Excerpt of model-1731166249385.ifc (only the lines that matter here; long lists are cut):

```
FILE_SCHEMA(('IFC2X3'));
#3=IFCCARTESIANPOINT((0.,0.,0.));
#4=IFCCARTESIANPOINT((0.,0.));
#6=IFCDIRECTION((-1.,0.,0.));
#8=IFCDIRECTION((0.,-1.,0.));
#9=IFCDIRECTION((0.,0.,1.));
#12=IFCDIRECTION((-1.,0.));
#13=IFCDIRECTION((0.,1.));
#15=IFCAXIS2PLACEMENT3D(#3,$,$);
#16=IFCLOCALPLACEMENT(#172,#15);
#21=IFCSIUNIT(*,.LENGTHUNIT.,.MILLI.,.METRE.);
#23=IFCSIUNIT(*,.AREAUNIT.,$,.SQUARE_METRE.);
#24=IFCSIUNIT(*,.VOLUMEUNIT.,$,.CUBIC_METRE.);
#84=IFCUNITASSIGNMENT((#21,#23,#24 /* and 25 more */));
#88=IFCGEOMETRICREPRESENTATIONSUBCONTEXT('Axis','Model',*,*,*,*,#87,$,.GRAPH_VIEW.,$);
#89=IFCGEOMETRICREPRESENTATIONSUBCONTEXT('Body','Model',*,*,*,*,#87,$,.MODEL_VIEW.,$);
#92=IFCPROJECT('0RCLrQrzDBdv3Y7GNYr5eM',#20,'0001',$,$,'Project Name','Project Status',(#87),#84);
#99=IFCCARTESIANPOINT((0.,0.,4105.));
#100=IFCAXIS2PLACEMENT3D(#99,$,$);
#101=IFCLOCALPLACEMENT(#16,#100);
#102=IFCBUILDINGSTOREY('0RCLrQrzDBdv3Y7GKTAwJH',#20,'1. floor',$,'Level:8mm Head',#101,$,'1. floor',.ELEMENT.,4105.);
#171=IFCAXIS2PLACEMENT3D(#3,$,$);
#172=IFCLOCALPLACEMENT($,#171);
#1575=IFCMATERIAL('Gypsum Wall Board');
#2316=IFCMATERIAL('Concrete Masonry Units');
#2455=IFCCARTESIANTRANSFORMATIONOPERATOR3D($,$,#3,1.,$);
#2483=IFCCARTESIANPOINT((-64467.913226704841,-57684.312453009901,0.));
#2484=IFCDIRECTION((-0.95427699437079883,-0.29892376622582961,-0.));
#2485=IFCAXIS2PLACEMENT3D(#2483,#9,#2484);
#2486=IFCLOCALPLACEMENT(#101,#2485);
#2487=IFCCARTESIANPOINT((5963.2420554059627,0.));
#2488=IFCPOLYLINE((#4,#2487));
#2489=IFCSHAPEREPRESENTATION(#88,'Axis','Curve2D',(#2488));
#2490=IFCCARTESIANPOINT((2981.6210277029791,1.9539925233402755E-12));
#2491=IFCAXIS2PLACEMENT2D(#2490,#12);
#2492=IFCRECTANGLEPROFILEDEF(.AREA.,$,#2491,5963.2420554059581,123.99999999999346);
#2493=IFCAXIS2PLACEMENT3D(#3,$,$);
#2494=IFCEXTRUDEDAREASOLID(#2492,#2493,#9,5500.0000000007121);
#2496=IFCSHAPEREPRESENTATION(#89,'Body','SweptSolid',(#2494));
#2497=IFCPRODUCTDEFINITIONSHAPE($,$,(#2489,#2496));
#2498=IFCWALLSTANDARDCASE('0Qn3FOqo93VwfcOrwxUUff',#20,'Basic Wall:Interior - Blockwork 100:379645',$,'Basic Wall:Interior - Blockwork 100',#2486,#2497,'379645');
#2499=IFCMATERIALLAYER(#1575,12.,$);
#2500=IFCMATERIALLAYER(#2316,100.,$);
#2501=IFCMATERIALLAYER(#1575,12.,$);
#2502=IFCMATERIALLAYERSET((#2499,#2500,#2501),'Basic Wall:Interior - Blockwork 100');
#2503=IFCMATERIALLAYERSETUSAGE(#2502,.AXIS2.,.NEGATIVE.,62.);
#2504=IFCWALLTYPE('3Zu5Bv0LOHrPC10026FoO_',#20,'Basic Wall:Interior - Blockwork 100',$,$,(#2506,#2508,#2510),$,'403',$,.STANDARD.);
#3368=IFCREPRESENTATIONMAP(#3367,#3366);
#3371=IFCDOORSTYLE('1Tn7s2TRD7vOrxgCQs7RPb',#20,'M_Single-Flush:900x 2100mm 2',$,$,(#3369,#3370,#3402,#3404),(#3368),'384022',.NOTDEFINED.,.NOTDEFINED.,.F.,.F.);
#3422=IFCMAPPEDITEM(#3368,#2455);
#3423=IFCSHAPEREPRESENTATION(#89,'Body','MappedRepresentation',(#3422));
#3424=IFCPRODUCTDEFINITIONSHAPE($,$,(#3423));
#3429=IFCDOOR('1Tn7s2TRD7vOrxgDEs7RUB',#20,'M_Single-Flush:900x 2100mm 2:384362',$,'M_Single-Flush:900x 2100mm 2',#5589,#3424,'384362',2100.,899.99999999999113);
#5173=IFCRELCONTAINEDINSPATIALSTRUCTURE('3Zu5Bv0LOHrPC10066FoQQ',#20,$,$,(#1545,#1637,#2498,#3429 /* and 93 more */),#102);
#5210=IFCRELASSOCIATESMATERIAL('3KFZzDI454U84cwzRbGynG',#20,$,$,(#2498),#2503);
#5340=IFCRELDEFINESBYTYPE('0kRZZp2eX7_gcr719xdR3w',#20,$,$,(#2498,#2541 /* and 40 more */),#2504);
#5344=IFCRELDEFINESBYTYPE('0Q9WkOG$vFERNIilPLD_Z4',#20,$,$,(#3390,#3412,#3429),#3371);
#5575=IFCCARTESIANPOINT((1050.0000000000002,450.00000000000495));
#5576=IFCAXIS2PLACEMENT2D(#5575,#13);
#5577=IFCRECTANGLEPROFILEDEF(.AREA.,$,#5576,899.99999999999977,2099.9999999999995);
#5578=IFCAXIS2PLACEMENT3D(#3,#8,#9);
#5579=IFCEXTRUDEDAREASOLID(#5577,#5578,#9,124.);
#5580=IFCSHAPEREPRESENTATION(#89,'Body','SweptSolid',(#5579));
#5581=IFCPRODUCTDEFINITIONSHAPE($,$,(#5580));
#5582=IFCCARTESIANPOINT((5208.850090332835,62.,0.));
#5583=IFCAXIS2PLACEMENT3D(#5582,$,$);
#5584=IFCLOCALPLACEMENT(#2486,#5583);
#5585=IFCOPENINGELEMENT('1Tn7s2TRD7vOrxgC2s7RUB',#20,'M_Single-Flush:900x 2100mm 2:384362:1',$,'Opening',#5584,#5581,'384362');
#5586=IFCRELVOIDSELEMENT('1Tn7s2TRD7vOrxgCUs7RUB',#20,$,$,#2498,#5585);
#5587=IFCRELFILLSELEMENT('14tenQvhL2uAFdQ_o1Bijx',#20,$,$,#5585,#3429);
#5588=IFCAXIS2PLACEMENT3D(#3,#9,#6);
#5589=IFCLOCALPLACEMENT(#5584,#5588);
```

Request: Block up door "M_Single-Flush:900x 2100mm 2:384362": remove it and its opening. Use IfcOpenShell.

```python
import ifcopenshell
import ifcopenshell.api.feature
import ifcopenshell.api.root
import ifcopenshell.geom
import ifcopenshell.util.shape

model = ifcopenshell.open("model-1731166249385.ifc")
settings = ifcopenshell.geom.settings()


def volume(element):
    """Net volume in cubic metres, openings subtracted."""
    shape = ifcopenshell.geom.create_shape(settings, element)
    return ifcopenshell.util.shape.get_volume(shape.geometry)


door = model.by_guid("1Tn7s2TRD7vOrxgDEs7RUB")
opening = door.FillsVoids[0].RelatingOpeningElement
wall = opening.VoidsElements[0].RelatingBuildingElement
before = volume(wall)

ifcopenshell.api.root.remove_product(model, product=door)
ifcopenshell.api.feature.remove_feature(model, feature=opening)

after = volume(wall)

print(f"wall volume {before:.3f} -> {after:.3f} m3")

model.write("model-1731166249385_v2.ifc")
```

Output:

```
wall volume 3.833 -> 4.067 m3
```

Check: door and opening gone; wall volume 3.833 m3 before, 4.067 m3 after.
